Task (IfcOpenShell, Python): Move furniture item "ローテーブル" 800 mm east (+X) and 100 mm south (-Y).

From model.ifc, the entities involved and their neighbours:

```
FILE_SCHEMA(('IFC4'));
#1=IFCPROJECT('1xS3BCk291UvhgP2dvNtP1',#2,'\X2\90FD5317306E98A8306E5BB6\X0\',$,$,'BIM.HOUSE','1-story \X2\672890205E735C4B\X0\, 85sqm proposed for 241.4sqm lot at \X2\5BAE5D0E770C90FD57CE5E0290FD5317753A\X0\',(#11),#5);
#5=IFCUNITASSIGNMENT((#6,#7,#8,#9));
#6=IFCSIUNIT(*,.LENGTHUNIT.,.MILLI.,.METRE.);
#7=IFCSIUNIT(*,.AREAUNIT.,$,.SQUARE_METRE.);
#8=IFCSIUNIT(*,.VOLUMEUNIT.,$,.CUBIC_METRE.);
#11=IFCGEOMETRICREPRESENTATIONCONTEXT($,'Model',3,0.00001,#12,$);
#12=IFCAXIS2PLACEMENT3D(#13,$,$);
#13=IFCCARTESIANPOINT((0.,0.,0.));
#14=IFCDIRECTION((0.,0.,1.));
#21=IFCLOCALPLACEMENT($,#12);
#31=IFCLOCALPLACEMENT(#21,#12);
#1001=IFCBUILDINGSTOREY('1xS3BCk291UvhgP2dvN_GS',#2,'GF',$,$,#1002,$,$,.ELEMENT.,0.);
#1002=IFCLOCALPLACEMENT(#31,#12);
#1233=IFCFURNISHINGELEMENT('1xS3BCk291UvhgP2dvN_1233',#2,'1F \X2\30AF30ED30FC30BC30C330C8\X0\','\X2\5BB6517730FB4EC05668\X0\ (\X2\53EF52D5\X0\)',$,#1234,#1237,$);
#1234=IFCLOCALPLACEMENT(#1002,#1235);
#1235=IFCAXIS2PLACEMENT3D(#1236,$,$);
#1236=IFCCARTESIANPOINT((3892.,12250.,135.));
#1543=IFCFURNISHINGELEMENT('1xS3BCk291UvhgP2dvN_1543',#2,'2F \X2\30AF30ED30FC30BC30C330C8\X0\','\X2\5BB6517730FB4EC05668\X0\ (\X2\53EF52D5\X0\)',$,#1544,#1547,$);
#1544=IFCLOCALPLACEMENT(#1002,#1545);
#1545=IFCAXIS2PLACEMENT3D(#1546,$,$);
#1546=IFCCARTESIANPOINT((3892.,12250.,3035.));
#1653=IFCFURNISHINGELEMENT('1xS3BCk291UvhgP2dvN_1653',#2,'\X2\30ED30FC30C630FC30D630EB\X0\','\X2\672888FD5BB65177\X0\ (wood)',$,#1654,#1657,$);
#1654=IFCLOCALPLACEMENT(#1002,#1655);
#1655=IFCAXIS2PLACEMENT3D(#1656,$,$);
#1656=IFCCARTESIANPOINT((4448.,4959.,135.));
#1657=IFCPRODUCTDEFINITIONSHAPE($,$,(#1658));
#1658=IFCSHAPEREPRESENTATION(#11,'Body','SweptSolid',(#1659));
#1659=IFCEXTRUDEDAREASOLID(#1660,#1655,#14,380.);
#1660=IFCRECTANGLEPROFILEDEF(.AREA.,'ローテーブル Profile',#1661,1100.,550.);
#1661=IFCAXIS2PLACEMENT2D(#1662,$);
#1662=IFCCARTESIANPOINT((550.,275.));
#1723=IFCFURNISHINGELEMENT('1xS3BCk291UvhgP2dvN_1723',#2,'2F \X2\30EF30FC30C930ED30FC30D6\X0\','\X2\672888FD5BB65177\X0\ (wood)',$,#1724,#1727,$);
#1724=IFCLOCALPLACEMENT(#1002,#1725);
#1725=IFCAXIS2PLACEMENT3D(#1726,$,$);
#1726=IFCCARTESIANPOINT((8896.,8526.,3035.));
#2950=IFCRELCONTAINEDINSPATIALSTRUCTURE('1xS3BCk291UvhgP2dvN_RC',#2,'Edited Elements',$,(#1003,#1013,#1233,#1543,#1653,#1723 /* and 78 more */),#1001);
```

```python
import ifcopenshell
import ifcopenshell.api.geometry
import ifcopenshell.util.placement

model = ifcopenshell.open("model.ifc")

item = model.by_guid("1xS3BCk291UvhgP2dvN_1653")
matrix = ifcopenshell.util.placement.get_local_placement(item.ObjectPlacement)
matrix[0, 3] += 800.0
matrix[1, 3] -= 100.0
ifcopenshell.api.geometry.edit_object_placement(model, product=item, matrix=matrix, is_si=False)

print(ifcopenshell.util.placement.get_local_placement(item.ObjectPlacement).round(3) + 0.0)

model.write("model_rev.ifc")
```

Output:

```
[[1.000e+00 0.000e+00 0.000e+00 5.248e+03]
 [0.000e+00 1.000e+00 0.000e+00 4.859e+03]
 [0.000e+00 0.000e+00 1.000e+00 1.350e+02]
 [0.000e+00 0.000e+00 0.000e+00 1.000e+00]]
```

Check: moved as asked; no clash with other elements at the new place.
